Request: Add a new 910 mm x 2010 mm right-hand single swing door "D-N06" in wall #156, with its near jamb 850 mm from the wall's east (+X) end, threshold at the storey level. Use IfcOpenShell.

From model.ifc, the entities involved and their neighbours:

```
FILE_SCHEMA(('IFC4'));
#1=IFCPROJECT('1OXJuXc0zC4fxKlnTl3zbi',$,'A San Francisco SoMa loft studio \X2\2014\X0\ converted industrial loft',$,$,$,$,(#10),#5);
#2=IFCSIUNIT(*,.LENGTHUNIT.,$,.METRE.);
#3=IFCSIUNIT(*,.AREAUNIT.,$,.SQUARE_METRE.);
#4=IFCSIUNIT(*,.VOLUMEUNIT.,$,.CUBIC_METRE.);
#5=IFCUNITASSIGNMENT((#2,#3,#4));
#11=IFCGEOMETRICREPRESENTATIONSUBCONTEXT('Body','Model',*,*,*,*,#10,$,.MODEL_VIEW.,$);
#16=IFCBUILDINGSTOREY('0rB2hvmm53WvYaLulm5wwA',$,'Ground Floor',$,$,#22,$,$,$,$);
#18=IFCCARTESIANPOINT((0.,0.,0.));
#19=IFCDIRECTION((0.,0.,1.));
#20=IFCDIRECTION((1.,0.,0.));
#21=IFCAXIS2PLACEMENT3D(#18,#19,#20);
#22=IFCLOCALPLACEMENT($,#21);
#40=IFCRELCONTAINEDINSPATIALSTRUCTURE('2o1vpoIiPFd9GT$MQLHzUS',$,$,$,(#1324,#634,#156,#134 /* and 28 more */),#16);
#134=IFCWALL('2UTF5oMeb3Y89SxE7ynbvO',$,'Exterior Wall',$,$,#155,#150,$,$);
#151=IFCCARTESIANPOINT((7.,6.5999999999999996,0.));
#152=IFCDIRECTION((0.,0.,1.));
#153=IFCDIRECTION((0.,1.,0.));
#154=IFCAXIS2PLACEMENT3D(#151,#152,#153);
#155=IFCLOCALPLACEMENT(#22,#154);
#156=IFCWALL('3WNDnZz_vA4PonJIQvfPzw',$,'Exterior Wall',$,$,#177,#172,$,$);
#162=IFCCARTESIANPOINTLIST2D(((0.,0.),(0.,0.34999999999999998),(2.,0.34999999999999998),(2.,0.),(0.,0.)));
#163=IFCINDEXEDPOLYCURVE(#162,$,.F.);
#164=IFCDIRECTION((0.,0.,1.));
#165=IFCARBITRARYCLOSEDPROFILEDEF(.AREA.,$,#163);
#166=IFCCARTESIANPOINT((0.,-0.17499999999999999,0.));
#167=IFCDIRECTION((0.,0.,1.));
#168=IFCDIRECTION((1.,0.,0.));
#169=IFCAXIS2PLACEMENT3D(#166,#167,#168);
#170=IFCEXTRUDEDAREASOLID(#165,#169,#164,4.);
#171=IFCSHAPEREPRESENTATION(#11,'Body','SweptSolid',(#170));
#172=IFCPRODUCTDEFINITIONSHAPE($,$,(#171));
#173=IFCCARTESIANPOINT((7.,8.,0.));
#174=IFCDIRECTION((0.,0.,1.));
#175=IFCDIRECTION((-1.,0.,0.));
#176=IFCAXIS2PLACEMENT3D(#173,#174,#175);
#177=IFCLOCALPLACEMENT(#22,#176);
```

```python
import numpy as np
import ifcopenshell
import ifcopenshell.api.feature
import ifcopenshell.api.geometry
import ifcopenshell.api.root
import ifcopenshell.api.spatial
import ifcopenshell.geom
import ifcopenshell.util.element
import ifcopenshell.util.placement
import ifcopenshell.util.representation
import ifcopenshell.util.shape
import ifcopenshell.util.unit

model = ifcopenshell.open("model.ifc")
unit_scale = ifcopenshell.util.unit.calculate_unit_scale(model)
settings = ifcopenshell.geom.settings()


def volume(element):
    """Net volume in cubic metres, openings subtracted."""
    shape = ifcopenshell.geom.create_shape(settings, element)
    return ifcopenshell.util.shape.get_volume(shape.geometry)


wall = model.by_guid("3WNDnZz_vA4PonJIQvfPzw")
storey = ifcopenshell.util.element.get_container(wall, ifc_class="IfcBuildingStorey")
context = ifcopenshell.util.representation.get_context(model, "Model", "Body", "MODEL_VIEW")
before = volume(wall)

width, height, from_end, sill = 0.91, 2.01, 0.85, 0.0  # metres

# The wall runs along its own X axis, and the end named is its -X end.
wall_shape = ifcopenshell.geom.create_shape(settings, wall)
x, y, z = ifcopenshell.util.shape.get_vertices(wall_shape.geometry).T
start = x.min() + from_end
face, thickness = float(y.min()), float(y.max() - y.min())
wall_matrix = ifcopenshell.util.placement.get_local_placement(wall.ObjectPlacement)
level = ifcopenshell.util.placement.get_local_placement(storey.ObjectPlacement)[2, 3]


def in_wall(x, y):
    """Placement at x, y metres in the wall's axes, at sill height."""
    matrix = wall_matrix.copy()
    matrix[:, 3] = wall_matrix @ np.array([x / unit_scale, y / unit_scale, 0.0, 1.0])
    matrix[2, 3] = level + sill / unit_scale
    return matrix


# Opening: a box that overshoots both wall faces by 50 mm.
opening = ifcopenshell.api.root.create_entity(model, ifc_class="IfcOpeningElement", predefined_type="OPENING")
box = ifcopenshell.api.geometry.add_wall_representation(
    model, context=context, length=width, height=height, thickness=thickness + 0.1
)
ifcopenshell.api.geometry.assign_representation(model, product=opening, representation=box)
ifcopenshell.api.geometry.edit_object_placement(model, product=opening, matrix=in_wall(start, face - 0.05), is_si=False)
ifcopenshell.api.feature.add_feature(model, feature=opening, element=wall)

door = ifcopenshell.api.root.create_entity(model, ifc_class="IfcDoor", name="D-N06", predefined_type="DOOR")
door.OverallWidth, door.OverallHeight = width / unit_scale, height / unit_scale
door.OperationType = "SINGLE_SWING_RIGHT"
body = ifcopenshell.api.geometry.add_door_representation(
    model,
    context=context,
    overall_width=door.OverallWidth,
    overall_height=door.OverallHeight,
    operation_type="SINGLE_SWING_RIGHT",
    lining_properties={"LiningDepth": thickness / unit_scale, "ThresholdDepth": thickness / unit_scale},
)
ifcopenshell.api.geometry.assign_representation(model, product=door, representation=body)
ifcopenshell.api.spatial.assign_container(model, products=[door], relating_structure=storey)
ifcopenshell.api.feature.add_filling(model, opening=opening, element=door)

# The lining spans the wall, so the door starts at the wall face.
ifcopenshell.api.geometry.edit_object_placement(model, product=door, matrix=in_wall(start, face), is_si=False)

after = volume(wall)

print(f"wall volume {before:.3f} -> {after:.3f} m3")

model.write("model-out.ifc")
```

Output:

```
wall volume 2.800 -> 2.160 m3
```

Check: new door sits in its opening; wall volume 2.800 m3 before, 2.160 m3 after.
